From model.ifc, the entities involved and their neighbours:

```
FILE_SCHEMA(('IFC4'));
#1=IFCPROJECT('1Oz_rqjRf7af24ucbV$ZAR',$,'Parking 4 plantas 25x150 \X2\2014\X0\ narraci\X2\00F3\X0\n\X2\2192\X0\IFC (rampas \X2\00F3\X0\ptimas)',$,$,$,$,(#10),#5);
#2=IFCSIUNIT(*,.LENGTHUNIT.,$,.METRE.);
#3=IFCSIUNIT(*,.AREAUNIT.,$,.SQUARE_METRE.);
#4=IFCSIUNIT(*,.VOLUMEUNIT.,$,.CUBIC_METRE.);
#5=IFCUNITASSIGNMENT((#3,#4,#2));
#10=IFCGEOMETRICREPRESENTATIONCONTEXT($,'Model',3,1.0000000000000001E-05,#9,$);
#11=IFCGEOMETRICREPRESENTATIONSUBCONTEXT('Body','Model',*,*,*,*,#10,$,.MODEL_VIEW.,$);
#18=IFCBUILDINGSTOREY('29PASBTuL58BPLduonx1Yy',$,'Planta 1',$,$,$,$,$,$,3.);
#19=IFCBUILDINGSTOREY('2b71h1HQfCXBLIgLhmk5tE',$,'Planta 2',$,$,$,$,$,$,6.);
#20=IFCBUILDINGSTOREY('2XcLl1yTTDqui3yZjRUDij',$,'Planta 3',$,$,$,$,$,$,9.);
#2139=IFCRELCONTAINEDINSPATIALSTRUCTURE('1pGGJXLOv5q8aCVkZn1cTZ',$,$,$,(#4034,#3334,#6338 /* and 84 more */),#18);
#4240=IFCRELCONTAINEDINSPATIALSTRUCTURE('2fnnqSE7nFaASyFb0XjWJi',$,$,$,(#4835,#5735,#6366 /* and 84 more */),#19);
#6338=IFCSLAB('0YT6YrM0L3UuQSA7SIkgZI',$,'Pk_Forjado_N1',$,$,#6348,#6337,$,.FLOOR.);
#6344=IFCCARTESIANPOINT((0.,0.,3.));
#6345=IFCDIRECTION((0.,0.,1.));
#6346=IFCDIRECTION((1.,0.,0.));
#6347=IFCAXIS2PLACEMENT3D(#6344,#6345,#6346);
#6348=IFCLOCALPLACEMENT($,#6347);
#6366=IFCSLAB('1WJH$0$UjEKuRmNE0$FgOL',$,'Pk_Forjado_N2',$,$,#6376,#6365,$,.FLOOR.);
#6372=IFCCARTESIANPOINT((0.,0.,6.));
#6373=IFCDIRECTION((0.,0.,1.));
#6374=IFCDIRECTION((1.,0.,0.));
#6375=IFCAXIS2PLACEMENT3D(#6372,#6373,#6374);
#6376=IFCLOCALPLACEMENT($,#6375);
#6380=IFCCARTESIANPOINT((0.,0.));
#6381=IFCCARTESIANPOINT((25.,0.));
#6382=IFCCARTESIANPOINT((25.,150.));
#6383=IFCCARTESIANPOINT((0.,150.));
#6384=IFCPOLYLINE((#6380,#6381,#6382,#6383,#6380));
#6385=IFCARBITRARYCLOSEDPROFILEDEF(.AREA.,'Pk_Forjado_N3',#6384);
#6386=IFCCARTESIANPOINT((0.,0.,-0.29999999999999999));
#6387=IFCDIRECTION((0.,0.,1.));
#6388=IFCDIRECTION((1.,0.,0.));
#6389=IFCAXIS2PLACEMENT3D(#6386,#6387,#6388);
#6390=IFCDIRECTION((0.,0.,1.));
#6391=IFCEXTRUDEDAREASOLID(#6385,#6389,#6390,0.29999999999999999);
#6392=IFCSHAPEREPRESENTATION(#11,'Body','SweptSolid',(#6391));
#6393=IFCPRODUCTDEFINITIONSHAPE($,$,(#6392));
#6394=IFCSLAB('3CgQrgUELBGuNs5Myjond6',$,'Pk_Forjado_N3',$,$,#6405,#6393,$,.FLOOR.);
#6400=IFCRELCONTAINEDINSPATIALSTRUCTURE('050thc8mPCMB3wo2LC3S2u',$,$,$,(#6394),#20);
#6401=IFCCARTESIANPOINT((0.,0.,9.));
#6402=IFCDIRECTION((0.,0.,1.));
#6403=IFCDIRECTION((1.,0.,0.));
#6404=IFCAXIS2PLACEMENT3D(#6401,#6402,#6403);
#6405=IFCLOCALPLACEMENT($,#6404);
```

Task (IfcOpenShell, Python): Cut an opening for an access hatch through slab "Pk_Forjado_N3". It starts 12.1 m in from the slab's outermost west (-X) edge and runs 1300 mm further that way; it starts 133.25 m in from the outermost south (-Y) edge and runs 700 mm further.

```python
import numpy as np
import ifcopenshell
import ifcopenshell.api.feature
import ifcopenshell.api.geometry
import ifcopenshell.api.root
import ifcopenshell.geom
import ifcopenshell.util.placement
import ifcopenshell.util.representation
import ifcopenshell.util.shape
import ifcopenshell.util.unit

model = ifcopenshell.open("model.ifc")
unit_scale = ifcopenshell.util.unit.calculate_unit_scale(model)
settings = ifcopenshell.geom.settings()


def volume(element):
    """Net volume in cubic metres, openings subtracted."""
    shape = ifcopenshell.geom.create_shape(settings, element)
    return ifcopenshell.util.shape.get_volume(shape.geometry)


slab = model.by_guid("3CgQrgUELBGuNs5Myjond6")
before = volume(slab)

# Extent in the slab's own axes, in metres. The edges named are its -X and -Y sides.
slab_shape = ifcopenshell.geom.create_shape(settings, slab)
vertices = ifcopenshell.util.shape.get_vertices(slab_shape.geometry)
x_min, y_min, bottom = vertices.min(axis=0)
top = vertices[:, 2].max()

opening = ifcopenshell.api.root.create_entity(model, ifc_class="IfcOpeningElement", name="Access hatch opening", predefined_type="OPENING")
context = ifcopenshell.util.representation.get_context(model, "Model", "Body", "MODEL_VIEW")
width, depth = 1.3, 0.7
outline = [(0.0, 0.0), (width, 0.0), (width, depth), (0.0, depth), (0.0, 0.0)]
# Overshoot both faces by 50 mm so the cut is clean.
shape = ifcopenshell.api.geometry.add_slab_representation(
    model, context=context, depth=top - bottom + 0.1, polyline=outline
)
ifcopenshell.api.geometry.assign_representation(model, product=opening, representation=shape)

matrix = ifcopenshell.util.placement.get_local_placement(slab.ObjectPlacement)
matrix[:, 3] = matrix @ np.append(np.array([x_min + 12.1, y_min + 133.25, bottom - 0.05]) / unit_scale, 1.0)
ifcopenshell.api.geometry.edit_object_placement(model, product=opening, matrix=matrix, is_si=False)
ifcopenshell.api.feature.add_feature(model, feature=opening, element=slab)

after = volume(slab)

print(f"slab volume {before:.3f} -> {after:.3f} m3")

model.write("model_edited.ifc")
```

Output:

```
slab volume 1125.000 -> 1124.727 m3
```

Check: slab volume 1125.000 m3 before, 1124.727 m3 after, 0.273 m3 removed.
